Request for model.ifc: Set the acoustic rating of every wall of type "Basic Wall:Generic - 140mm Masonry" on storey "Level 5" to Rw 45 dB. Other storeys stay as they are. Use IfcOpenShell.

First a look at what the model holds.

```python
import ifcopenshell
import ifcopenshell.util.element

model = ifcopenshell.open("model.ifc")
print(model.schema)
storey = next(s for s in model.by_type("IfcBuildingStorey") if s.Name == "Level 5")
walls = [e for e in ifcopenshell.util.element.get_decomposition(storey) if e.is_a("IfcWall")]
seen = {}
for e in walls:
    element_type = ifcopenshell.util.element.get_type(e)
    key = (element_type.Name if element_type != e and element_type else None, ifcopenshell.util.element.get_pset(e, "Pset_WallCommon", "AcousticRating"))
    seen[key] = seen.get(key, 0) + 1
for (name, value), count in sorted(seen.items(), key=str):
    print(count, "x", name, "|", value)
```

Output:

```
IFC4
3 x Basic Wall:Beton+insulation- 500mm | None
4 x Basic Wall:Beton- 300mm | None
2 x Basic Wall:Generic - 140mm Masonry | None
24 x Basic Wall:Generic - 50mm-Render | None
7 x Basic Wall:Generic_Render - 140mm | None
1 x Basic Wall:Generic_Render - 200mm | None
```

```python
import ifcopenshell
import ifcopenshell.api.pset
import ifcopenshell.util.element

model = ifcopenshell.open("model.ifc")

storey = next(s for s in model.by_type("IfcBuildingStorey") if s.Name == "Level 5")
walls = [e for e in ifcopenshell.util.element.get_decomposition(storey) if e.is_a("IfcWall")]

count = 0
for e in walls:
    element_type = ifcopenshell.util.element.get_type(e)
    if element_type in (None, e) or element_type.Name != "Basic Wall:Generic - 140mm Masonry":
        continue
    # add_pset returns the element's existing set when there is one.
    pset = ifcopenshell.api.pset.add_pset(model, product=e, name="Pset_WallCommon")
    ifcopenshell.api.pset.edit_pset(model, pset=pset, properties={"AcousticRating": "Rw 45 dB"})
    count += 1

print(count, "walls updated")

model.write("model_v2.ifc")
```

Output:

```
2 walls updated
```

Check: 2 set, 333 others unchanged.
